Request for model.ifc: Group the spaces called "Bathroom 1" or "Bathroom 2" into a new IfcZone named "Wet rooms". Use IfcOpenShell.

First a look at what the model holds.

```python
import ifcopenshell

model = ifcopenshell.open("model.ifc")
print(model.schema)
seen = {}
for space in model.by_type("IfcSpace"):
    seen[space.LongName] = seen.get(space.LongName, 0) + 1
for name, count in sorted(seen.items(), key=str):
    print(count, "x", name)
print("zones:", [z.Name for z in model.by_type("IfcZone")][:20])
```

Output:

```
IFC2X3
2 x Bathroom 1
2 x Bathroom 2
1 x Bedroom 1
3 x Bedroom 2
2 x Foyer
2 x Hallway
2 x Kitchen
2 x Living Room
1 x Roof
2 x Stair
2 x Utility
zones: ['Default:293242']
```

```python
import ifcopenshell
import ifcopenshell.api.group
import ifcopenshell.api.root

model = ifcopenshell.open("model.ifc")

names = {"Bathroom 1", "Bathroom 2"}
spaces = [s for s in model.by_type("IfcSpace") if s.LongName in names]

zone = ifcopenshell.api.root.create_entity(model, ifc_class="IfcZone", name="Wet rooms")
ifcopenshell.api.group.assign_group(model, products=spaces, group=zone)
print(len(spaces), "spaces in", zone.Name)

model.write("model_edited.ifc")
```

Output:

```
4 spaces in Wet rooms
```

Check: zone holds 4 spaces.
